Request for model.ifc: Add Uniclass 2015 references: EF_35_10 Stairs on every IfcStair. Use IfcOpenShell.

First a look at what the model holds.

```python
import ifcopenshell

model = ifcopenshell.open("model.ifc")
print(model.schema)
print("classifications:", [c.Name for c in model.by_type("IfcClassification")])
for ifc_class in ("IfcDoor", "IfcRoof", "IfcStair", "IfcWall", "IfcWindow"):
    print(ifc_class, len(model.by_type(ifc_class)))
```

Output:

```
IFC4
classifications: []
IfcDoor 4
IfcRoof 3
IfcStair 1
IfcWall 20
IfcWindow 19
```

```python
import ifcopenshell
import ifcopenshell.api.classification

model = ifcopenshell.open("model.ifc")

system = ifcopenshell.api.classification.add_classification(model, classification="Uniclass 2015")

codes = {
    "IfcStair": ("EF_35_10", "Stairs"),
}
for ifc_class, (code, name) in codes.items():
    products = model.by_type(ifc_class)
    ifcopenshell.api.classification.add_reference(
        model, products=products, classification=system, identification=code, name=name
    )
    print(code, len(products))

model.write("model_updated.ifc")
```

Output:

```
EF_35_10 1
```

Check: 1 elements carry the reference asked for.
